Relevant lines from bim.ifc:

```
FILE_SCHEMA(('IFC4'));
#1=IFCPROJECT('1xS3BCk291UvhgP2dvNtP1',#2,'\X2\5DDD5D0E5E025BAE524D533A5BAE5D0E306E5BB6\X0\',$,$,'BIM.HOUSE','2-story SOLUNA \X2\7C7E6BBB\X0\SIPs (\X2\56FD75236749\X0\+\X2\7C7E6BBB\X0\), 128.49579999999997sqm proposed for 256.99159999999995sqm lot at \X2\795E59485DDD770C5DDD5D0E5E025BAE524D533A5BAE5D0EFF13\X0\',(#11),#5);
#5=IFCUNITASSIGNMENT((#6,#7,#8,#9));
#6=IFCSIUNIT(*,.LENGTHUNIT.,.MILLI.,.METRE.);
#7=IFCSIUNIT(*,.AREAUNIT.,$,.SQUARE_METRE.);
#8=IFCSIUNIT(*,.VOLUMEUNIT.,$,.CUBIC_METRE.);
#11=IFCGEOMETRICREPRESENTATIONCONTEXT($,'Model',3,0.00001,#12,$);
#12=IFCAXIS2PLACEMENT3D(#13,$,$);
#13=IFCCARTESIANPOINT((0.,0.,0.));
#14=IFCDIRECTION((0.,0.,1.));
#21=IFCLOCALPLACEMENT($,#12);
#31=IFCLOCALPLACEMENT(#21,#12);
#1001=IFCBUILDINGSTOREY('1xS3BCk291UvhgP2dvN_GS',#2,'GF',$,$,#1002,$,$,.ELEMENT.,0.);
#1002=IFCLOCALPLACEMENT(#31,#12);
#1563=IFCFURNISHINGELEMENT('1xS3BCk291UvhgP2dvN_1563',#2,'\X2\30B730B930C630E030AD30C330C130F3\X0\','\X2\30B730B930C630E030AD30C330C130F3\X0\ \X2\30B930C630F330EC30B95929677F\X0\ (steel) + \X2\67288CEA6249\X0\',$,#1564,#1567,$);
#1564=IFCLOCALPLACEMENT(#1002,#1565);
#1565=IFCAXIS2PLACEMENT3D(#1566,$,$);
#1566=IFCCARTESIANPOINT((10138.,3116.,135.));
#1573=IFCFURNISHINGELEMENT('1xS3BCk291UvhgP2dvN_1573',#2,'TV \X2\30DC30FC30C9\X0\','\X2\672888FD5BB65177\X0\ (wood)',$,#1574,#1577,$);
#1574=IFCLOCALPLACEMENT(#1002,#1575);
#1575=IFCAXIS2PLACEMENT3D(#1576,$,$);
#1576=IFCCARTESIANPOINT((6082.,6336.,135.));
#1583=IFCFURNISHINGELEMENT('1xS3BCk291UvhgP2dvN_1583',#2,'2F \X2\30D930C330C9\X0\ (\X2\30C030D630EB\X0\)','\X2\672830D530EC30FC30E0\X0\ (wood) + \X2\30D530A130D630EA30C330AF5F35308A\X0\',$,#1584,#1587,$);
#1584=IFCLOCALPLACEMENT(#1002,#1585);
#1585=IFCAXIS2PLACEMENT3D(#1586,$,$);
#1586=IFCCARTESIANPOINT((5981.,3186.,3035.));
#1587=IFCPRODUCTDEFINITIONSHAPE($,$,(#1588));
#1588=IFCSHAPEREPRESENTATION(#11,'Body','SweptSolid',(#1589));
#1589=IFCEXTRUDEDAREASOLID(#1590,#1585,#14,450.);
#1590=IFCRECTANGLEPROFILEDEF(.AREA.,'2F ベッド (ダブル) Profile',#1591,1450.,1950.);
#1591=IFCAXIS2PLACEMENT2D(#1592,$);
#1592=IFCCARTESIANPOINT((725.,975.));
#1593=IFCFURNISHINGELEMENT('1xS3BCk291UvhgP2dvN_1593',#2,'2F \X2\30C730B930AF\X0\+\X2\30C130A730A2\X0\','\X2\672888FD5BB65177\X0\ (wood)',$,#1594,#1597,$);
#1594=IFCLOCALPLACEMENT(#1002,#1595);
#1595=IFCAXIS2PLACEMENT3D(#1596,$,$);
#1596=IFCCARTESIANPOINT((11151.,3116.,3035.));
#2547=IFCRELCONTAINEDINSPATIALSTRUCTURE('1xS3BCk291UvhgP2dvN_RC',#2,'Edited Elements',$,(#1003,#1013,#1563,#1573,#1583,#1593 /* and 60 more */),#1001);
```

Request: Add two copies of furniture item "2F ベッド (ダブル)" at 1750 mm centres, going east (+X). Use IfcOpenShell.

```python
import numpy as np
import ifcopenshell
import ifcopenshell.api.geometry
import ifcopenshell.api.root
import ifcopenshell.util.element
import ifcopenshell.util.placement

model = ifcopenshell.open("bim.ifc")


def reuse_history(source, copy):
    """copy_class also copies each property set's owner history, people and application; keep the originals."""
    for rel in copy.IsDefinedBy:
        if rel.is_a("IfcRelDefinesByProperties") and (history := rel.RelatingPropertyDefinition.OwnerHistory):
            rel.RelatingPropertyDefinition.OwnerHistory = source.OwnerHistory
            ifcopenshell.util.element.remove_deep2(model, history)


source = model.by_guid("1xS3BCk291UvhgP2dvN_1583")
base = ifcopenshell.util.placement.get_local_placement(source.ObjectPlacement)
step = np.array([1.0, 0.0, 0.0]) * 1750.0

for i in range(1, 3):
    copy = ifcopenshell.api.root.copy_class(model, product=source)
    copy.Representation = ifcopenshell.util.element.copy_deep(
        model, source.Representation, exclude=["IfcGeometricRepresentationContext", "IfcRepresentationMap"]
    )
    reuse_history(source, copy)
    matrix = base.copy()
    matrix[:3, 3] += i * step
    print("added at", matrix[:3, 3].round(3) + 0.0)
    ifcopenshell.api.geometry.edit_object_placement(model, product=copy, matrix=matrix, is_si=False)

model.write("bim_rev.ifc")
```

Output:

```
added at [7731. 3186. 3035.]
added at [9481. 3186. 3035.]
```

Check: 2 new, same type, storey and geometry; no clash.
